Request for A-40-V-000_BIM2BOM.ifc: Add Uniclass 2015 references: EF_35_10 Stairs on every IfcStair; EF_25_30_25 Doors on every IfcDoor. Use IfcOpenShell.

First a look at what the model holds.

```python
import ifcopenshell

model = ifcopenshell.open("A-40-V-000_BIM2BOM.ifc")
print(model.schema)
print("classifications:", [c.Name for c in model.by_type("IfcClassification")])
for ifc_class in ("IfcDoor", "IfcRoof", "IfcStair", "IfcWall", "IfcWindow"):
    print(ifc_class, len(model.by_type(ifc_class)))
```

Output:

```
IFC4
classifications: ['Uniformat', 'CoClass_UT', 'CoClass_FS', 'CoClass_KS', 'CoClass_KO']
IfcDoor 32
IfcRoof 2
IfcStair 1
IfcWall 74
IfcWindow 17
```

```python
import ifcopenshell
import ifcopenshell.api.classification

model = ifcopenshell.open("A-40-V-000_BIM2BOM.ifc")

system = ifcopenshell.api.classification.add_classification(model, classification="Uniclass 2015")

codes = {
    "IfcStair": ("EF_35_10", "Stairs"),
    "IfcDoor": ("EF_25_30_25", "Doors"),
}
for ifc_class, (code, name) in codes.items():
    products = model.by_type(ifc_class)
    ifcopenshell.api.classification.add_reference(
        model, products=products, classification=system, identification=code, name=name
    )
    print(code, len(products))

model.write("A-40-V-000_BIM2BOM_rev.ifc")
```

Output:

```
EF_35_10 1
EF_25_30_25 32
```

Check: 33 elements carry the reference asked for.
